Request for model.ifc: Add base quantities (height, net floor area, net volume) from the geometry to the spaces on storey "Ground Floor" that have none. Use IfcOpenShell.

First a look at what the model holds.

```python
import ifcopenshell
import ifcopenshell.util.element
import ifcopenshell.util.unit

model = ifcopenshell.open("model.ifc")
print(model.schema)
for unit_type in ("LENGTHUNIT", "AREAUNIT", "VOLUMEUNIT"):
    print(unit_type, ifcopenshell.util.unit.calculate_unit_scale(model, unit_type))
storey = next(s for s in model.by_type("IfcBuildingStorey") if s.Name == "Ground Floor")
spaces = [e for e in ifcopenshell.util.element.get_decomposition(storey) if e.is_a("IfcSpace")]
for e in sorted(spaces, key=lambda e: e.id()):
    print(e.id(), e.is_a(), e.Name, list(ifcopenshell.util.element.get_psets(e, qtos_only=True)), sep=" | ")
```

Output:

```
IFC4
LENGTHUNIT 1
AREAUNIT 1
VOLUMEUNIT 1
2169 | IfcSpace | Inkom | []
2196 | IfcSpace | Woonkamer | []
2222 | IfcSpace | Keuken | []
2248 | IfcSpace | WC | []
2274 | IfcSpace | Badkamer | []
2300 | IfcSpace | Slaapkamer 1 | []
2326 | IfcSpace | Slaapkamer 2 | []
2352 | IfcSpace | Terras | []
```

```python
import ifcopenshell
import ifcopenshell.api.pset
import ifcopenshell.geom
import ifcopenshell.util.element
import ifcopenshell.util.shape
import ifcopenshell.util.unit

model = ifcopenshell.open("model.ifc")
unit_scale = ifcopenshell.util.unit.calculate_unit_scale(model)
area_scale = ifcopenshell.util.unit.calculate_unit_scale(model, "AREAUNIT")
volume_scale = ifcopenshell.util.unit.calculate_unit_scale(model, "VOLUMEUNIT")
settings = ifcopenshell.geom.settings()

storey = next(s for s in model.by_type("IfcBuildingStorey") if s.Name == "Ground Floor")
spaces = [e for e in ifcopenshell.util.element.get_decomposition(storey) if e.is_a("IfcSpace")]

for e in sorted(spaces, key=lambda e: e.id()):
    if ifcopenshell.util.element.get_psets(e, qtos_only=True, should_inherit=False):
        continue
    # Geometry comes back in metres, in the element's own axes.
    shape = ifcopenshell.geom.create_shape(settings, e)
    values = {
        "Height": ifcopenshell.util.shape.get_z(shape.geometry) / unit_scale,
        "NetFloorArea": ifcopenshell.util.shape.get_footprint_area(shape.geometry) / area_scale,
        "NetVolume": ifcopenshell.util.shape.get_volume(shape.geometry) / volume_scale,
    }
    qto = ifcopenshell.api.pset.add_qto(model, product=e, name="Qto_SpaceBaseQuantities")
    ifcopenshell.api.pset.edit_qto(model, qto=qto, properties=values)
    print(e.id(), {k: round(v, 3) for k, v in values.items()})

model.write("model_edited.ifc")
```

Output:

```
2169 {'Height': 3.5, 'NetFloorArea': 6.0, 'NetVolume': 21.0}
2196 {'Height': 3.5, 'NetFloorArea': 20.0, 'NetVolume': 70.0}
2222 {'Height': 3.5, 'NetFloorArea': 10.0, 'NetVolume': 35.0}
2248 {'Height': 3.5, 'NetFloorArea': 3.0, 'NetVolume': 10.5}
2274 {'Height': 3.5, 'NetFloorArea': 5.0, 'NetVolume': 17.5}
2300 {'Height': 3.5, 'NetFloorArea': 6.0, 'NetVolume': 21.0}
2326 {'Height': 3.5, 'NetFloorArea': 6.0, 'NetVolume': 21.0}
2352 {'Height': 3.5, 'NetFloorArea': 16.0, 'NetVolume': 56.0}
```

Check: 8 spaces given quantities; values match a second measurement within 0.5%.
